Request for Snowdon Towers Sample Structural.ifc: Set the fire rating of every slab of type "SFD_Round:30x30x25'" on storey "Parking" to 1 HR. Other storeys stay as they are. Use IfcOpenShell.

First a look at what the model holds.

```python
import ifcopenshell
import ifcopenshell.util.element

model = ifcopenshell.open("Snowdon Towers Sample Structural.ifc")
print(model.schema)
storey = next(s for s in model.by_type("IfcBuildingStorey") if s.Name == "Parking")
slabs = [e for e in ifcopenshell.util.element.get_decomposition(storey) if e.is_a("IfcSlab")]
seen = {}
for e in slabs:
    element_type = ifcopenshell.util.element.get_type(e)
    key = (element_type.Name if element_type != e and element_type else None, ifcopenshell.util.element.get_pset(e, "Pset_SlabCommon", "FireRating"))
    seen[key] = seen.get(key, 0) + 1
for (name, value), count in sorted(seen.items(), key=str):
    print(count, "x", name, "|", value)
```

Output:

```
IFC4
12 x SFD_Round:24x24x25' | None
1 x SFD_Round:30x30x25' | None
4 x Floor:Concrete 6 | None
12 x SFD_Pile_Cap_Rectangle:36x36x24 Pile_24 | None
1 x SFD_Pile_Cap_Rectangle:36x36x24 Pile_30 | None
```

```python
import ifcopenshell
import ifcopenshell.api.pset
import ifcopenshell.util.element

model = ifcopenshell.open("Snowdon Towers Sample Structural.ifc")

storey = next(s for s in model.by_type("IfcBuildingStorey") if s.Name == "Parking")
slabs = [e for e in ifcopenshell.util.element.get_decomposition(storey) if e.is_a("IfcSlab")]

count = 0
for e in slabs:
    element_type = ifcopenshell.util.element.get_type(e)
    if element_type in (None, e) or element_type.Name != "SFD_Round:30x30x25'":
        continue
    # add_pset returns the element's existing set when there is one.
    pset = ifcopenshell.api.pset.add_pset(model, product=e, name="Pset_SlabCommon")
    ifcopenshell.api.pset.edit_pset(model, pset=pset, properties={"FireRating": "1 HR"})
    count += 1

print(count, "slabs updated")

model.write("Snowdon Towers Sample Structural_edited.ifc")
```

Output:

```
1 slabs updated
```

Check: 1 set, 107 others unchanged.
